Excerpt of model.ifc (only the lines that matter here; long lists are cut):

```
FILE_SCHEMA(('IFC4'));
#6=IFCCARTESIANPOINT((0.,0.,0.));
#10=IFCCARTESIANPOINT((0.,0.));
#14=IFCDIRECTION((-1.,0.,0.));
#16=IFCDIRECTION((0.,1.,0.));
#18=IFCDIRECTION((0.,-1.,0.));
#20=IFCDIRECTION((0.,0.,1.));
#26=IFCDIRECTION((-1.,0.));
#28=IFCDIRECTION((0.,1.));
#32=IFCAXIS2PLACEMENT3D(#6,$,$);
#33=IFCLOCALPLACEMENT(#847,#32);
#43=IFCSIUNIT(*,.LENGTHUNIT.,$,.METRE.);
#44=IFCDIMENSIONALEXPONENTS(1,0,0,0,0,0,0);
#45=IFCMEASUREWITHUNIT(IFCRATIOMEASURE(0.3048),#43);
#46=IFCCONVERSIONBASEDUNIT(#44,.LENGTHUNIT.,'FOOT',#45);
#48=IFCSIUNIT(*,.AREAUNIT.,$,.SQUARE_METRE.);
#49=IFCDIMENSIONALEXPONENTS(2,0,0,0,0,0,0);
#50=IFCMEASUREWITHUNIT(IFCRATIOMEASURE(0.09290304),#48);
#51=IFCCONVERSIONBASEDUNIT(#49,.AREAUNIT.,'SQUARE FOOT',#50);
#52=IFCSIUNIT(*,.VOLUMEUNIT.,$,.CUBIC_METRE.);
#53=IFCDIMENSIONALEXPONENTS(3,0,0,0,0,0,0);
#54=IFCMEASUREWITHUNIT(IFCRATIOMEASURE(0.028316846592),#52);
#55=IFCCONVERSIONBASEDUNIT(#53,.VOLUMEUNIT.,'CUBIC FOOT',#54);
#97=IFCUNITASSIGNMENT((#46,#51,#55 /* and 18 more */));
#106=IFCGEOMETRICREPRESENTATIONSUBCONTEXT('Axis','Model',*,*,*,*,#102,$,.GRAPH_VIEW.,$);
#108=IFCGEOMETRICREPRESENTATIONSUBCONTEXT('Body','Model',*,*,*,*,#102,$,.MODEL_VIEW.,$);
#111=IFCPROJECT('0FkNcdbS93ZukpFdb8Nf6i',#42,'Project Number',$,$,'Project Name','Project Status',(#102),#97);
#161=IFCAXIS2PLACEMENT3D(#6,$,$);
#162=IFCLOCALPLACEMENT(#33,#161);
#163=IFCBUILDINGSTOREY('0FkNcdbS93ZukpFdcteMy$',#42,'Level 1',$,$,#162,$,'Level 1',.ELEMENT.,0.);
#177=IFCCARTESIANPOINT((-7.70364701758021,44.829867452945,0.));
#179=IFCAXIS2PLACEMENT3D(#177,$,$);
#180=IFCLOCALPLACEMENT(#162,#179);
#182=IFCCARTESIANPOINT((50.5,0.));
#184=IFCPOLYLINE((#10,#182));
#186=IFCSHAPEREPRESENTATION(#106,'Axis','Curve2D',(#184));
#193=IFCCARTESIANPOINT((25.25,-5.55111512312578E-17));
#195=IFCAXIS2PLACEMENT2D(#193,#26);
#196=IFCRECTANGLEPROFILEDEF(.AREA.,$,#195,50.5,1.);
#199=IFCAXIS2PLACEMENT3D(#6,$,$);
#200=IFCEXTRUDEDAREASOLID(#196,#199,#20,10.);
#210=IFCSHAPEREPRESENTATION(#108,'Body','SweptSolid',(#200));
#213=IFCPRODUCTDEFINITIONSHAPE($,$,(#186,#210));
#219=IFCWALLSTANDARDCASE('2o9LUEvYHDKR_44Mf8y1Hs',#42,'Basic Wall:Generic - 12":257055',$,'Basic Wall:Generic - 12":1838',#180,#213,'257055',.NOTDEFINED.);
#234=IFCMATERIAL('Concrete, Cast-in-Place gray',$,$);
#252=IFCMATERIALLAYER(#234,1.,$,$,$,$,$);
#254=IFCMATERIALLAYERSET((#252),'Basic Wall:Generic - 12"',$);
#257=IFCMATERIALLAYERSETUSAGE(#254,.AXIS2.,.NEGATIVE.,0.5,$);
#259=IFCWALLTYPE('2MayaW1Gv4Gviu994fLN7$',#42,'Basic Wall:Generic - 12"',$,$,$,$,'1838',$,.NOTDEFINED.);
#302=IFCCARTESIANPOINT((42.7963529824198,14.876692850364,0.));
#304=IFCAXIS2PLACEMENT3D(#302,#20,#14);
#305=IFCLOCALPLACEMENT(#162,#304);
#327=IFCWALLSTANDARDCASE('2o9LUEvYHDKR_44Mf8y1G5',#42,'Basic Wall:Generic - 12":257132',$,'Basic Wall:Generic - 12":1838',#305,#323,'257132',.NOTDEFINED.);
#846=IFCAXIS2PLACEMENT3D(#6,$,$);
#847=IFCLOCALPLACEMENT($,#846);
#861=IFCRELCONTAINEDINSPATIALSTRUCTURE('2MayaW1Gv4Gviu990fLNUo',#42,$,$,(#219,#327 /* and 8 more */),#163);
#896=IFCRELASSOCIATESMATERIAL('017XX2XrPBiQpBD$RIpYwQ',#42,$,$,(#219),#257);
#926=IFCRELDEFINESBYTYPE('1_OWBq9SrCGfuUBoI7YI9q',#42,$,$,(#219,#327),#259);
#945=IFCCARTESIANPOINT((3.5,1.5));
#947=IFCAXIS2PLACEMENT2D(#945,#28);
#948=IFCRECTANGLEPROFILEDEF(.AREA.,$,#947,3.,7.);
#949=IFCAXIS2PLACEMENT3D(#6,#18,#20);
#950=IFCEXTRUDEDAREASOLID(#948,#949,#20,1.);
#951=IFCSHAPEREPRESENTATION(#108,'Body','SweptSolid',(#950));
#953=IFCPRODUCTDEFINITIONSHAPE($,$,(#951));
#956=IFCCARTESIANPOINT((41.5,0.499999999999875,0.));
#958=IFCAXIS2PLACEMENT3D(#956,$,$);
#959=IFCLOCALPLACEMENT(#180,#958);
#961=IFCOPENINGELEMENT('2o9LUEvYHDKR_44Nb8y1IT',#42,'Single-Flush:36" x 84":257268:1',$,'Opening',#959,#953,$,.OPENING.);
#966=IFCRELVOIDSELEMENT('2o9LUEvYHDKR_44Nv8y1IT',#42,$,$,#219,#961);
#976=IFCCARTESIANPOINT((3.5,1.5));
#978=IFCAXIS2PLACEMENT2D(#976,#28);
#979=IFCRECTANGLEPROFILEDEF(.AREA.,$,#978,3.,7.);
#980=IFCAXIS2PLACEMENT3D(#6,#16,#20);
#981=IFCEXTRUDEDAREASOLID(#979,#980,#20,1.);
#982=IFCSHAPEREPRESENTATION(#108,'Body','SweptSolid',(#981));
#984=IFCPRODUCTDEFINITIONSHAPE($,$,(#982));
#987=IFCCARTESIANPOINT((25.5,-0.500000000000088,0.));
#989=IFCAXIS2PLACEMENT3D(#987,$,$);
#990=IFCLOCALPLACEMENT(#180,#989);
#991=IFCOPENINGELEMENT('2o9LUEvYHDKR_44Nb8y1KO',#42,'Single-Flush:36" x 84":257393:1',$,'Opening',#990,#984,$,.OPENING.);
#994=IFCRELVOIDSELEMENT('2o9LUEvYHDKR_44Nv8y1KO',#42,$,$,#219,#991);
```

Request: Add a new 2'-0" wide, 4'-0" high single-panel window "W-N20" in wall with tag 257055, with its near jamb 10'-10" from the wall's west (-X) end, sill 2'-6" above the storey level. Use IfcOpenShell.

```python
import numpy as np
import ifcopenshell
import ifcopenshell.api.feature
import ifcopenshell.api.geometry
import ifcopenshell.api.root
import ifcopenshell.api.spatial
import ifcopenshell.geom
import ifcopenshell.util.element
import ifcopenshell.util.placement
import ifcopenshell.util.representation
import ifcopenshell.util.shape
import ifcopenshell.util.unit

model = ifcopenshell.open("model.ifc")
unit_scale = ifcopenshell.util.unit.calculate_unit_scale(model)
settings = ifcopenshell.geom.settings()


def volume(element):
    """Net volume in cubic metres, openings subtracted."""
    shape = ifcopenshell.geom.create_shape(settings, element)
    return ifcopenshell.util.shape.get_volume(shape.geometry)


wall = model.by_guid("2o9LUEvYHDKR_44Mf8y1Hs")
storey = ifcopenshell.util.element.get_container(wall, ifc_class="IfcBuildingStorey")
context = ifcopenshell.util.representation.get_context(model, "Model", "Body", "MODEL_VIEW")
before = volume(wall)

width, height, from_end, sill = 0.6096, 1.2192, 3.302, 0.762  # metres

# The wall runs along its own X axis, and the end named is its -X end.
wall_shape = ifcopenshell.geom.create_shape(settings, wall)
x, y, z = ifcopenshell.util.shape.get_vertices(wall_shape.geometry).T
start = x.min() + from_end
face, thickness = float(y.min()), float(y.max() - y.min())
wall_matrix = ifcopenshell.util.placement.get_local_placement(wall.ObjectPlacement)
level = ifcopenshell.util.placement.get_local_placement(storey.ObjectPlacement)[2, 3]


def in_wall(x, y):
    """Placement at x, y metres in the wall's axes, at sill height."""
    matrix = wall_matrix.copy()
    matrix[:, 3] = wall_matrix @ np.array([x / unit_scale, y / unit_scale, 0.0, 1.0])
    matrix[2, 3] = level + sill / unit_scale
    return matrix


# Opening: a box that overshoots both wall faces by 50 mm.
opening = ifcopenshell.api.root.create_entity(model, ifc_class="IfcOpeningElement", predefined_type="OPENING")
box = ifcopenshell.api.geometry.add_wall_representation(
    model, context=context, length=width, height=height, thickness=thickness + 0.1
)
ifcopenshell.api.geometry.assign_representation(model, product=opening, representation=box)
ifcopenshell.api.geometry.edit_object_placement(model, product=opening, matrix=in_wall(start, face - 0.05), is_si=False)
ifcopenshell.api.feature.add_feature(model, feature=opening, element=wall)

window = ifcopenshell.api.root.create_entity(model, ifc_class="IfcWindow", name="W-N20", predefined_type="WINDOW")
window.OverallWidth, window.OverallHeight = width / unit_scale, height / unit_scale
window.PartitioningType = "SINGLE_PANEL"
body = ifcopenshell.api.geometry.add_window_representation(
    model,
    context=context,
    overall_width=window.OverallWidth,
    overall_height=window.OverallHeight,
    partition_type="SINGLE_PANEL",
)
ifcopenshell.api.geometry.assign_representation(model, product=window, representation=body)
ifcopenshell.api.spatial.assign_container(model, products=[window], relating_structure=storey)
ifcopenshell.api.feature.add_filling(model, opening=opening, element=window)

# Centre the window in the wall's thickness.
ifcopenshell.api.geometry.edit_object_placement(model, product=window, matrix=in_wall(start, face), is_si=False)
window_shape = ifcopenshell.geom.create_shape(settings, window)
depth = ifcopenshell.util.shape.get_vertices(window_shape.geometry)[:, 1]
offset = face + thickness / 2 - (depth.min() + depth.max()) / 2
ifcopenshell.api.geometry.edit_object_placement(model, product=window, matrix=in_wall(start, offset), is_si=False)

after = volume(wall)

print(f"wall volume {before:.3f} -> {after:.3f} m3")

model.write("model_rev.ifc")
```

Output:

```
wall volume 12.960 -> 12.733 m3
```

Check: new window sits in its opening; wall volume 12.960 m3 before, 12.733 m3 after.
